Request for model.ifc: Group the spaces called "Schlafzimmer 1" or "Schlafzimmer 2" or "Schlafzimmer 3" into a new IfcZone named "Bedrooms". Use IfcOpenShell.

First a look at what the model holds.

```python
import ifcopenshell

model = ifcopenshell.open("model.ifc")
print(model.schema)
seen = {}
for space in model.by_type("IfcSpace"):
    seen[space.LongName] = seen.get(space.LongName, 0) + 1
for name, count in sorted(seen.items(), key=str):
    print(count, "x", name)
print("zones:", [z.Name for z in model.by_type("IfcZone")][:20])
```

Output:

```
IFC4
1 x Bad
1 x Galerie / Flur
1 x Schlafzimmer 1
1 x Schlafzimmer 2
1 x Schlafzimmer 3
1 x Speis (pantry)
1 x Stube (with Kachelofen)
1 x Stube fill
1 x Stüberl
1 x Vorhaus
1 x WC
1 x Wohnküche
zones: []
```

```python
import ifcopenshell
import ifcopenshell.api.group
import ifcopenshell.api.root

model = ifcopenshell.open("model.ifc")

names = {"Schlafzimmer 1", "Schlafzimmer 2", "Schlafzimmer 3"}
spaces = [s for s in model.by_type("IfcSpace") if s.LongName in names]

zone = ifcopenshell.api.root.create_entity(model, ifc_class="IfcZone", name="Bedrooms")
ifcopenshell.api.group.assign_group(model, products=spaces, group=zone)
print(len(spaces), "spaces in", zone.Name)

model.write("model-out.ifc")
```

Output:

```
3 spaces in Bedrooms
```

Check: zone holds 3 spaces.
